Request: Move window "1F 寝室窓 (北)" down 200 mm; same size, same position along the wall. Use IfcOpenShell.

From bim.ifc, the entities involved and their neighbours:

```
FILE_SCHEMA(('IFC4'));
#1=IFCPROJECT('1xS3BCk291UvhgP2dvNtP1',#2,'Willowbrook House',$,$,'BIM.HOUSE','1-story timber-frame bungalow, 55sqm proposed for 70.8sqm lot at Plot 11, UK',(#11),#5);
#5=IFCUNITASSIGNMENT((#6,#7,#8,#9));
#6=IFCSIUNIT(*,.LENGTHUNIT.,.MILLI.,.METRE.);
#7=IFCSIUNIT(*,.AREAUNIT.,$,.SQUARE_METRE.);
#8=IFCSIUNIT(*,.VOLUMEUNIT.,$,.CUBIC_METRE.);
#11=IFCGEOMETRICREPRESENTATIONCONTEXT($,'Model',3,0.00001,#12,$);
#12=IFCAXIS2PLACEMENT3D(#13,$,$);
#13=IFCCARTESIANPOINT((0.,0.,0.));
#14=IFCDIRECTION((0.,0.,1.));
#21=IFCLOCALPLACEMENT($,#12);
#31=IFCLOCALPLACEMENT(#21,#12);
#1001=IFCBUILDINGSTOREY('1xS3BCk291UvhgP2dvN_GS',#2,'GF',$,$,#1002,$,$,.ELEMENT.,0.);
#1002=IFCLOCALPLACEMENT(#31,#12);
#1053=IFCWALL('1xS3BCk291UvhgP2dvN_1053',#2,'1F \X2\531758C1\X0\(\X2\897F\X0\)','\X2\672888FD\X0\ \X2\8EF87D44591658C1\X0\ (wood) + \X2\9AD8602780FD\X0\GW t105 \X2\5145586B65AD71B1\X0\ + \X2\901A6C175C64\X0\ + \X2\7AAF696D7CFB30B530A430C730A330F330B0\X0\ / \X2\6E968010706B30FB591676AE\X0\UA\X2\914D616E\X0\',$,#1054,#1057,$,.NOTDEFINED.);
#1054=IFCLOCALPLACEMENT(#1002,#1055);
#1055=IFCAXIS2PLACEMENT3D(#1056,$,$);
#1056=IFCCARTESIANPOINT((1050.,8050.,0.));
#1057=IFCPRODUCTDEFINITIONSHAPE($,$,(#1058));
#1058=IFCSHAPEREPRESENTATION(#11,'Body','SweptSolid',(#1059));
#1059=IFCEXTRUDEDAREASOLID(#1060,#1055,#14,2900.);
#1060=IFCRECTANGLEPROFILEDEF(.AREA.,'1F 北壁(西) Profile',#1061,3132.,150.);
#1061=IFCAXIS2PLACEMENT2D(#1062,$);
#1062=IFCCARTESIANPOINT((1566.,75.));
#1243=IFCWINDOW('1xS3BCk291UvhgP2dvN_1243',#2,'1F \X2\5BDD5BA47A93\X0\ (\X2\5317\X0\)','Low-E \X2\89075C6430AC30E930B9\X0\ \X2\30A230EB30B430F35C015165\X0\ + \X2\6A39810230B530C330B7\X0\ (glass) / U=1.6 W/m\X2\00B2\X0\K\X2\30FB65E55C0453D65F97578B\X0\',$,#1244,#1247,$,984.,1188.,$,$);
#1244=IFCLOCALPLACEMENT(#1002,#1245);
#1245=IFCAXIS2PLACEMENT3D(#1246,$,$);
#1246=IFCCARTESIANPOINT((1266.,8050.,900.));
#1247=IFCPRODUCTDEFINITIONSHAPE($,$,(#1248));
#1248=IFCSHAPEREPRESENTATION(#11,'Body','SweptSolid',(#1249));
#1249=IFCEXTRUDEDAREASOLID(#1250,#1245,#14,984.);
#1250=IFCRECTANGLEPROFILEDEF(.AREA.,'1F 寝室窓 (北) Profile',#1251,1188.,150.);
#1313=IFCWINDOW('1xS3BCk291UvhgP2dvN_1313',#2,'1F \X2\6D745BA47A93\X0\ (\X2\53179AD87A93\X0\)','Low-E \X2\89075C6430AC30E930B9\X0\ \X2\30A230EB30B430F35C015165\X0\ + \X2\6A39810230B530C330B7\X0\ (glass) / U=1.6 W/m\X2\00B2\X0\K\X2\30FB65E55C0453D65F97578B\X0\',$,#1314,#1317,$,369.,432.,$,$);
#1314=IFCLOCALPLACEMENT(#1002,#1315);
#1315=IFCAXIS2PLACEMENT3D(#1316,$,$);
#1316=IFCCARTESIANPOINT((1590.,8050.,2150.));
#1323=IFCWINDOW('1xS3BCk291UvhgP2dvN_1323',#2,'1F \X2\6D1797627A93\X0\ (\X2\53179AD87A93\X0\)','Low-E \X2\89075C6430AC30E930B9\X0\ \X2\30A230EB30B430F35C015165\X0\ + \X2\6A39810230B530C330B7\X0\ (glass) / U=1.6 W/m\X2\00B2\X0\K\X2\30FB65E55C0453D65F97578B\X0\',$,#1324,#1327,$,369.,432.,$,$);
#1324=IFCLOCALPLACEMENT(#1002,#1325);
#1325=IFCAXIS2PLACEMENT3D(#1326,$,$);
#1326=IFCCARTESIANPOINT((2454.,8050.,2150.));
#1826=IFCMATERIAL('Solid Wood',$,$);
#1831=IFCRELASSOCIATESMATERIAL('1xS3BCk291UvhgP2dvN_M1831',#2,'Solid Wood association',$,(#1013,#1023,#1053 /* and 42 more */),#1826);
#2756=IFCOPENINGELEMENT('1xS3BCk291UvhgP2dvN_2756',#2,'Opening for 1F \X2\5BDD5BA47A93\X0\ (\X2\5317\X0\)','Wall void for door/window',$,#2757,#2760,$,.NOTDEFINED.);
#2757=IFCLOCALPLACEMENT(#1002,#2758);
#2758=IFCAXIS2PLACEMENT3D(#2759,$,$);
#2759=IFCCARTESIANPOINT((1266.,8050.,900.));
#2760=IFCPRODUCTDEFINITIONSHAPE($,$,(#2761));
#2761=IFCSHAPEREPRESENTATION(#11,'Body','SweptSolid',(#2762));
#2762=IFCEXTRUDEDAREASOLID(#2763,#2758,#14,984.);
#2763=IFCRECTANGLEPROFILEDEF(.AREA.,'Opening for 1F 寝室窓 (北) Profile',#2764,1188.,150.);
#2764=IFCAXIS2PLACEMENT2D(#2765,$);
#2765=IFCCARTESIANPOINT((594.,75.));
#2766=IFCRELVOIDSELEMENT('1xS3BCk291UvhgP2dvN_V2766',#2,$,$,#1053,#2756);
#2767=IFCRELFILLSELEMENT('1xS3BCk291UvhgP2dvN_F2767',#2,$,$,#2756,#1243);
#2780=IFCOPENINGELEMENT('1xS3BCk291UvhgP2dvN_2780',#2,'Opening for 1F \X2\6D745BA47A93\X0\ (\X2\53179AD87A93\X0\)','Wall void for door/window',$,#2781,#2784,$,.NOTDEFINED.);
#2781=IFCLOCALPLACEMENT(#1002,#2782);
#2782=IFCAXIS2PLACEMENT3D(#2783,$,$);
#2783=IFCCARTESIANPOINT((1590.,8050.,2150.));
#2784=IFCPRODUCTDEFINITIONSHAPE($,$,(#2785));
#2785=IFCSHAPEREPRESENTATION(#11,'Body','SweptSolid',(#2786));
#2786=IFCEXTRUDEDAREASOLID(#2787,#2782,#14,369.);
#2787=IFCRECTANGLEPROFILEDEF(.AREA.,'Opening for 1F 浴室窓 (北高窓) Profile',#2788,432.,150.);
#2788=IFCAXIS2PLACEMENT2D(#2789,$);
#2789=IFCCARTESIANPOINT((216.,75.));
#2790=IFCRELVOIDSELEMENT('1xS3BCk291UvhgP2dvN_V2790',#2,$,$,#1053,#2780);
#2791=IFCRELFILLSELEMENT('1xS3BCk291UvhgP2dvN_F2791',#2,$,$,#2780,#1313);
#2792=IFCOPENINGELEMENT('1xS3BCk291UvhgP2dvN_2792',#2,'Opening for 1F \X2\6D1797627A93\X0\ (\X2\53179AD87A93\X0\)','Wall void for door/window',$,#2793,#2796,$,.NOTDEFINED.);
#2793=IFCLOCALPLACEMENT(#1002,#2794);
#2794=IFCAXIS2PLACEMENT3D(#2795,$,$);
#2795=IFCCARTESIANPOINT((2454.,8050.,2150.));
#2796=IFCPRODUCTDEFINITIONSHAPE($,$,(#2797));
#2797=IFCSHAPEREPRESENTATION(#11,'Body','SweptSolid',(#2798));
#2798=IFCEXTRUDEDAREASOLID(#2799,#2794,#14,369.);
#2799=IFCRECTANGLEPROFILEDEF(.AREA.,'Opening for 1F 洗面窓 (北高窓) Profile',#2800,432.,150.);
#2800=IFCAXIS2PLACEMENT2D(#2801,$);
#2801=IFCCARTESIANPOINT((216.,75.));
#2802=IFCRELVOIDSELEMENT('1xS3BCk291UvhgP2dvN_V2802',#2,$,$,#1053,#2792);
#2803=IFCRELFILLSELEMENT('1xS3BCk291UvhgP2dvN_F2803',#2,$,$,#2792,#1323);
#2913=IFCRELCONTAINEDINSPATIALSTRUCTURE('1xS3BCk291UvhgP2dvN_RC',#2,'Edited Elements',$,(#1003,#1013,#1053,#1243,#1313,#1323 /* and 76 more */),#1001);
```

```python
import numpy as np
import ifcopenshell
import ifcopenshell.api.geometry
import ifcopenshell.util.placement
import ifcopenshell.util.unit

model = ifcopenshell.open("bim.ifc")
unit_scale = ifcopenshell.util.unit.calculate_unit_scale(model)

window = model.by_guid("1xS3BCk291UvhgP2dvN_1243")
opening = window.FillsVoids[0].RelatingOpeningElement
dz = -0.2 / unit_scale

shift = np.array([0.0, 0.0, dz])
# The window is not placed relative to its opening, so move both.
for product in (opening, window):
    matrix = ifcopenshell.util.placement.get_local_placement(product.ObjectPlacement)
    matrix[:3, 3] += shift
    ifcopenshell.api.geometry.edit_object_placement(model, product=product, matrix=matrix, is_si=False)

print(f"moved by {dz * unit_scale:+.3f} m")

model.write("bim_rev.ifc")
```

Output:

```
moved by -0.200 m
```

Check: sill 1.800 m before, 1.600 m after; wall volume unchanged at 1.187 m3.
